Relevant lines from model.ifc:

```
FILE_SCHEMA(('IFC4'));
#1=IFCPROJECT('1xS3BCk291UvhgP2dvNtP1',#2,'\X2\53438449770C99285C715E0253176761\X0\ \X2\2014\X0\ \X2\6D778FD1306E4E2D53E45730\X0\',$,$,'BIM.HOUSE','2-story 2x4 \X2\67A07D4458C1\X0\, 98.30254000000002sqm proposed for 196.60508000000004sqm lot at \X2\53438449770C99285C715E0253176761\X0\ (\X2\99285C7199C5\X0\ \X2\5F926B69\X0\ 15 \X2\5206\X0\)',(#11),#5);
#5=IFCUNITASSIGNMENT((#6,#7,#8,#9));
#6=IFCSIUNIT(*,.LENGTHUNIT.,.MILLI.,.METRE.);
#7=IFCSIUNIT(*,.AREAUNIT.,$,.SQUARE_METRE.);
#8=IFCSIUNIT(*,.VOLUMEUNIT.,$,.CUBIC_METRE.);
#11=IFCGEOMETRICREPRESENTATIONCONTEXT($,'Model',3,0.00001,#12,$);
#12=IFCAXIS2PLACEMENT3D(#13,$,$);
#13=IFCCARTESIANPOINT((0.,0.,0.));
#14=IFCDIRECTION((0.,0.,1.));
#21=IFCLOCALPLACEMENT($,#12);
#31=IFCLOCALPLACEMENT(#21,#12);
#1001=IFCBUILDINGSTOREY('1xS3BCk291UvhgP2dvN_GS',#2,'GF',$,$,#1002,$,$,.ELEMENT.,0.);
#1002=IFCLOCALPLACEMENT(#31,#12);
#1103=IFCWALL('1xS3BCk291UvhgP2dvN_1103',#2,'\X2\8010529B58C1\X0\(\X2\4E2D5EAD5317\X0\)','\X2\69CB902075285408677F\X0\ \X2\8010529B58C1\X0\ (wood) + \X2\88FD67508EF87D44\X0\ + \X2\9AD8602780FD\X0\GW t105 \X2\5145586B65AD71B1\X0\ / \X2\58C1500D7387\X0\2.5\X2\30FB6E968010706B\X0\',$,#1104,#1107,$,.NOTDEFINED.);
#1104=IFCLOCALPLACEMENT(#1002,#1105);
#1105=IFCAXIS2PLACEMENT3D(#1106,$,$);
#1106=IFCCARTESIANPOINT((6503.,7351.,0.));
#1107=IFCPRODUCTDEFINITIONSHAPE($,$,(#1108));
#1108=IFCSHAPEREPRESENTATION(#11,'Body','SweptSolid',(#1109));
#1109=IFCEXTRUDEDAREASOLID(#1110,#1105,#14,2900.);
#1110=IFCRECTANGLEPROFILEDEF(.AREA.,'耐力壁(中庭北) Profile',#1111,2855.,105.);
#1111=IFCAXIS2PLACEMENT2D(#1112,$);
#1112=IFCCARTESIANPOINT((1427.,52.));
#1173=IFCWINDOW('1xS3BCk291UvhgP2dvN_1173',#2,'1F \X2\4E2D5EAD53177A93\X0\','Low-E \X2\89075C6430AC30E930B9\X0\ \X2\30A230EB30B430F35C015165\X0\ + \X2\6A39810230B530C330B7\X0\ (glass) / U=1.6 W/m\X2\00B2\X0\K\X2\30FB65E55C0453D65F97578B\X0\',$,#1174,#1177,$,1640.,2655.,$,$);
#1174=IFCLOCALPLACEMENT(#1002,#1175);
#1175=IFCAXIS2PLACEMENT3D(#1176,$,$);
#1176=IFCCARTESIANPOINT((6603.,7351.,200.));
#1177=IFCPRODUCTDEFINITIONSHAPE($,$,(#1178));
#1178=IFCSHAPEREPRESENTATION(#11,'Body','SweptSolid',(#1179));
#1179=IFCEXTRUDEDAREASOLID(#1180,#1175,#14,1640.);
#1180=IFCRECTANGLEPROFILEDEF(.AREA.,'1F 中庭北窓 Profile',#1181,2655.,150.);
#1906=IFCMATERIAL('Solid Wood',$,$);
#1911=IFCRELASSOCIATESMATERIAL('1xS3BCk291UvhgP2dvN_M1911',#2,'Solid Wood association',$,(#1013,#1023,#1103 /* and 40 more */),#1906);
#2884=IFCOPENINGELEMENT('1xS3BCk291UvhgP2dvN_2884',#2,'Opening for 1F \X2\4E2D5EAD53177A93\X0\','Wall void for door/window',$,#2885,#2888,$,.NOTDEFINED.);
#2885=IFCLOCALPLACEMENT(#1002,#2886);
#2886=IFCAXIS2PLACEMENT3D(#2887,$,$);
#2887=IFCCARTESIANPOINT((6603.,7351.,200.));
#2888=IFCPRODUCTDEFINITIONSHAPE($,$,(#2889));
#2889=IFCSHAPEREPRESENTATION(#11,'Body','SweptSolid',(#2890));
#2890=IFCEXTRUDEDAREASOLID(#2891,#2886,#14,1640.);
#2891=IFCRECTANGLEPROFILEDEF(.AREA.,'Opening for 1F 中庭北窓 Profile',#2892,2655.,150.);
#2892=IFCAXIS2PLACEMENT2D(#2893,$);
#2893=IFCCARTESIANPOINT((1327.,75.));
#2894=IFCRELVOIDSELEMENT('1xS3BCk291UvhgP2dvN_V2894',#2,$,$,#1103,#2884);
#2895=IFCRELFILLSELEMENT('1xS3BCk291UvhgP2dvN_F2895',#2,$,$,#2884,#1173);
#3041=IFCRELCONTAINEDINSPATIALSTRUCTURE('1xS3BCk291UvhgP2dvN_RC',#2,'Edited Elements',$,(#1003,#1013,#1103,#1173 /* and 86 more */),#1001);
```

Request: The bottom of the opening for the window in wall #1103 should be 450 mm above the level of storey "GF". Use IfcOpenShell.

```python
import numpy as np
import ifcopenshell
import ifcopenshell.api.geometry
import ifcopenshell.geom
import ifcopenshell.util.element
import ifcopenshell.util.placement
import ifcopenshell.util.shape
import ifcopenshell.util.unit

model = ifcopenshell.open("model.ifc")
unit_scale = ifcopenshell.util.unit.calculate_unit_scale(model)

window = model.by_guid("1xS3BCk291UvhgP2dvN_1173")
opening = window.FillsVoids[0].RelatingOpeningElement
storey = ifcopenshell.util.element.get_container(window, ifc_class="IfcBuildingStorey")
level = ifcopenshell.util.placement.get_local_placement(storey.ObjectPlacement)[2, 3]

# The opening's origin need not be at the sill, so measure its lowest point.
shape = ifcopenshell.geom.create_shape(ifcopenshell.geom.settings(), opening)
bottom = ifcopenshell.util.shape.get_shape_bottom_elevation(shape, shape.geometry) / unit_scale
dz = level + 450.0 - bottom

shift = np.array([0.0, 0.0, dz])
# The window is not placed relative to its opening, so move both.
for product in (opening, window):
    matrix = ifcopenshell.util.placement.get_local_placement(product.ObjectPlacement)
    matrix[:3, 3] += shift
    ifcopenshell.api.geometry.edit_object_placement(model, product=product, matrix=matrix, is_si=False)

print(f"moved by {dz * unit_scale:+.3f} m")

model.write("model-out.ifc")
```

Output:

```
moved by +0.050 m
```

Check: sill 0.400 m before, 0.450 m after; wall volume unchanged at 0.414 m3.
